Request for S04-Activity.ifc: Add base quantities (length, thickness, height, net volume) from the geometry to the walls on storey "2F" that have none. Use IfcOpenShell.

First a look at what the model holds.

```python
import ifcopenshell
import ifcopenshell.util.element
import ifcopenshell.util.unit

model = ifcopenshell.open("S04-Activity.ifc")
print(model.schema)
for unit_type in ("LENGTHUNIT", "AREAUNIT", "VOLUMEUNIT"):
    print(unit_type, ifcopenshell.util.unit.calculate_unit_scale(model, unit_type))
storey = next(s for s in model.by_type("IfcBuildingStorey") if s.Name == "2F")
walls = [e for e in ifcopenshell.util.element.get_decomposition(storey) if e.is_a("IfcWall")]
for e in sorted(walls, key=lambda e: e.id()):
    print(e.id(), e.is_a(), e.Name, list(ifcopenshell.util.element.get_psets(e, qtos_only=True)), sep=" | ")
```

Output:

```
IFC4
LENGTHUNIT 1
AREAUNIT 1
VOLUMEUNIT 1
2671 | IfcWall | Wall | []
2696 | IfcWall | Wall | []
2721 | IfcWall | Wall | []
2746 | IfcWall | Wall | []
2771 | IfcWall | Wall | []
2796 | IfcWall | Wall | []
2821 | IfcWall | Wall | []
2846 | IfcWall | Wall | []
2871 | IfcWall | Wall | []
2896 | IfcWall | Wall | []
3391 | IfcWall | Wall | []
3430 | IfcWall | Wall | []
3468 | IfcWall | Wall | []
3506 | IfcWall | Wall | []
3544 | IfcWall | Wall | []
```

```python
import ifcopenshell
import ifcopenshell.api.pset
import ifcopenshell.geom
import ifcopenshell.util.element
import ifcopenshell.util.shape
import ifcopenshell.util.unit

model = ifcopenshell.open("S04-Activity.ifc")
unit_scale = ifcopenshell.util.unit.calculate_unit_scale(model)
volume_scale = ifcopenshell.util.unit.calculate_unit_scale(model, "VOLUMEUNIT")
settings = ifcopenshell.geom.settings()

storey = next(s for s in model.by_type("IfcBuildingStorey") if s.Name == "2F")
walls = [e for e in ifcopenshell.util.element.get_decomposition(storey) if e.is_a("IfcWall")]

for e in sorted(walls, key=lambda e: e.id()):
    if ifcopenshell.util.element.get_psets(e, qtos_only=True, should_inherit=False):
        continue
    # Geometry comes back in metres, in the element's own axes.
    shape = ifcopenshell.geom.create_shape(settings, e)
    values = {
        "Length": ifcopenshell.util.shape.get_x(shape.geometry) / unit_scale,
        "Width": ifcopenshell.util.shape.get_y(shape.geometry) / unit_scale,
        "Height": ifcopenshell.util.shape.get_z(shape.geometry) / unit_scale,
        "NetVolume": ifcopenshell.util.shape.get_volume(shape.geometry) / volume_scale,
    }
    qto = ifcopenshell.api.pset.add_qto(model, product=e, name="Qto_WallBaseQuantities")
    ifcopenshell.api.pset.edit_qto(model, qto=qto, properties=values)
    print(e.id(), {k: round(v, 3) for k, v in values.items()})

model.write("S04-Activity_rev.ifc")
```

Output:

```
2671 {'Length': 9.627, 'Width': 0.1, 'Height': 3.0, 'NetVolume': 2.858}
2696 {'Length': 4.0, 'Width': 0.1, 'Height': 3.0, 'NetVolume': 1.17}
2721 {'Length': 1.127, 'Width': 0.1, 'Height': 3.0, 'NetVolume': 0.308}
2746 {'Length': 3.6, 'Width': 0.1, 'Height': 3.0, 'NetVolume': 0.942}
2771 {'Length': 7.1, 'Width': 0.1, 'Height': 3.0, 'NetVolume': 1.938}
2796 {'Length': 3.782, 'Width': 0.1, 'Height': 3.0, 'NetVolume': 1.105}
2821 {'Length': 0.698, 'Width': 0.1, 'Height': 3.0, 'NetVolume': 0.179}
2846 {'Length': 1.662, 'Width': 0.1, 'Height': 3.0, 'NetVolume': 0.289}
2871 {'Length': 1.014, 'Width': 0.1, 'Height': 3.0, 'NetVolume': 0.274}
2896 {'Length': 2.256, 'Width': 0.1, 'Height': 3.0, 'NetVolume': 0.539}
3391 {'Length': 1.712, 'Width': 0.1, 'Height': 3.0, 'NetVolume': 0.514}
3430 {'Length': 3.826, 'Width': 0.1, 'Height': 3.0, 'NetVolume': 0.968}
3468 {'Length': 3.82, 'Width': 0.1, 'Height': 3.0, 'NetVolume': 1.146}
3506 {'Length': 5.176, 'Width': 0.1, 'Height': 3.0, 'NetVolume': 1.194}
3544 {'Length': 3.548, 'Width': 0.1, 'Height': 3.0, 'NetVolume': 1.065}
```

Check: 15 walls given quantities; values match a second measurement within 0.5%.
